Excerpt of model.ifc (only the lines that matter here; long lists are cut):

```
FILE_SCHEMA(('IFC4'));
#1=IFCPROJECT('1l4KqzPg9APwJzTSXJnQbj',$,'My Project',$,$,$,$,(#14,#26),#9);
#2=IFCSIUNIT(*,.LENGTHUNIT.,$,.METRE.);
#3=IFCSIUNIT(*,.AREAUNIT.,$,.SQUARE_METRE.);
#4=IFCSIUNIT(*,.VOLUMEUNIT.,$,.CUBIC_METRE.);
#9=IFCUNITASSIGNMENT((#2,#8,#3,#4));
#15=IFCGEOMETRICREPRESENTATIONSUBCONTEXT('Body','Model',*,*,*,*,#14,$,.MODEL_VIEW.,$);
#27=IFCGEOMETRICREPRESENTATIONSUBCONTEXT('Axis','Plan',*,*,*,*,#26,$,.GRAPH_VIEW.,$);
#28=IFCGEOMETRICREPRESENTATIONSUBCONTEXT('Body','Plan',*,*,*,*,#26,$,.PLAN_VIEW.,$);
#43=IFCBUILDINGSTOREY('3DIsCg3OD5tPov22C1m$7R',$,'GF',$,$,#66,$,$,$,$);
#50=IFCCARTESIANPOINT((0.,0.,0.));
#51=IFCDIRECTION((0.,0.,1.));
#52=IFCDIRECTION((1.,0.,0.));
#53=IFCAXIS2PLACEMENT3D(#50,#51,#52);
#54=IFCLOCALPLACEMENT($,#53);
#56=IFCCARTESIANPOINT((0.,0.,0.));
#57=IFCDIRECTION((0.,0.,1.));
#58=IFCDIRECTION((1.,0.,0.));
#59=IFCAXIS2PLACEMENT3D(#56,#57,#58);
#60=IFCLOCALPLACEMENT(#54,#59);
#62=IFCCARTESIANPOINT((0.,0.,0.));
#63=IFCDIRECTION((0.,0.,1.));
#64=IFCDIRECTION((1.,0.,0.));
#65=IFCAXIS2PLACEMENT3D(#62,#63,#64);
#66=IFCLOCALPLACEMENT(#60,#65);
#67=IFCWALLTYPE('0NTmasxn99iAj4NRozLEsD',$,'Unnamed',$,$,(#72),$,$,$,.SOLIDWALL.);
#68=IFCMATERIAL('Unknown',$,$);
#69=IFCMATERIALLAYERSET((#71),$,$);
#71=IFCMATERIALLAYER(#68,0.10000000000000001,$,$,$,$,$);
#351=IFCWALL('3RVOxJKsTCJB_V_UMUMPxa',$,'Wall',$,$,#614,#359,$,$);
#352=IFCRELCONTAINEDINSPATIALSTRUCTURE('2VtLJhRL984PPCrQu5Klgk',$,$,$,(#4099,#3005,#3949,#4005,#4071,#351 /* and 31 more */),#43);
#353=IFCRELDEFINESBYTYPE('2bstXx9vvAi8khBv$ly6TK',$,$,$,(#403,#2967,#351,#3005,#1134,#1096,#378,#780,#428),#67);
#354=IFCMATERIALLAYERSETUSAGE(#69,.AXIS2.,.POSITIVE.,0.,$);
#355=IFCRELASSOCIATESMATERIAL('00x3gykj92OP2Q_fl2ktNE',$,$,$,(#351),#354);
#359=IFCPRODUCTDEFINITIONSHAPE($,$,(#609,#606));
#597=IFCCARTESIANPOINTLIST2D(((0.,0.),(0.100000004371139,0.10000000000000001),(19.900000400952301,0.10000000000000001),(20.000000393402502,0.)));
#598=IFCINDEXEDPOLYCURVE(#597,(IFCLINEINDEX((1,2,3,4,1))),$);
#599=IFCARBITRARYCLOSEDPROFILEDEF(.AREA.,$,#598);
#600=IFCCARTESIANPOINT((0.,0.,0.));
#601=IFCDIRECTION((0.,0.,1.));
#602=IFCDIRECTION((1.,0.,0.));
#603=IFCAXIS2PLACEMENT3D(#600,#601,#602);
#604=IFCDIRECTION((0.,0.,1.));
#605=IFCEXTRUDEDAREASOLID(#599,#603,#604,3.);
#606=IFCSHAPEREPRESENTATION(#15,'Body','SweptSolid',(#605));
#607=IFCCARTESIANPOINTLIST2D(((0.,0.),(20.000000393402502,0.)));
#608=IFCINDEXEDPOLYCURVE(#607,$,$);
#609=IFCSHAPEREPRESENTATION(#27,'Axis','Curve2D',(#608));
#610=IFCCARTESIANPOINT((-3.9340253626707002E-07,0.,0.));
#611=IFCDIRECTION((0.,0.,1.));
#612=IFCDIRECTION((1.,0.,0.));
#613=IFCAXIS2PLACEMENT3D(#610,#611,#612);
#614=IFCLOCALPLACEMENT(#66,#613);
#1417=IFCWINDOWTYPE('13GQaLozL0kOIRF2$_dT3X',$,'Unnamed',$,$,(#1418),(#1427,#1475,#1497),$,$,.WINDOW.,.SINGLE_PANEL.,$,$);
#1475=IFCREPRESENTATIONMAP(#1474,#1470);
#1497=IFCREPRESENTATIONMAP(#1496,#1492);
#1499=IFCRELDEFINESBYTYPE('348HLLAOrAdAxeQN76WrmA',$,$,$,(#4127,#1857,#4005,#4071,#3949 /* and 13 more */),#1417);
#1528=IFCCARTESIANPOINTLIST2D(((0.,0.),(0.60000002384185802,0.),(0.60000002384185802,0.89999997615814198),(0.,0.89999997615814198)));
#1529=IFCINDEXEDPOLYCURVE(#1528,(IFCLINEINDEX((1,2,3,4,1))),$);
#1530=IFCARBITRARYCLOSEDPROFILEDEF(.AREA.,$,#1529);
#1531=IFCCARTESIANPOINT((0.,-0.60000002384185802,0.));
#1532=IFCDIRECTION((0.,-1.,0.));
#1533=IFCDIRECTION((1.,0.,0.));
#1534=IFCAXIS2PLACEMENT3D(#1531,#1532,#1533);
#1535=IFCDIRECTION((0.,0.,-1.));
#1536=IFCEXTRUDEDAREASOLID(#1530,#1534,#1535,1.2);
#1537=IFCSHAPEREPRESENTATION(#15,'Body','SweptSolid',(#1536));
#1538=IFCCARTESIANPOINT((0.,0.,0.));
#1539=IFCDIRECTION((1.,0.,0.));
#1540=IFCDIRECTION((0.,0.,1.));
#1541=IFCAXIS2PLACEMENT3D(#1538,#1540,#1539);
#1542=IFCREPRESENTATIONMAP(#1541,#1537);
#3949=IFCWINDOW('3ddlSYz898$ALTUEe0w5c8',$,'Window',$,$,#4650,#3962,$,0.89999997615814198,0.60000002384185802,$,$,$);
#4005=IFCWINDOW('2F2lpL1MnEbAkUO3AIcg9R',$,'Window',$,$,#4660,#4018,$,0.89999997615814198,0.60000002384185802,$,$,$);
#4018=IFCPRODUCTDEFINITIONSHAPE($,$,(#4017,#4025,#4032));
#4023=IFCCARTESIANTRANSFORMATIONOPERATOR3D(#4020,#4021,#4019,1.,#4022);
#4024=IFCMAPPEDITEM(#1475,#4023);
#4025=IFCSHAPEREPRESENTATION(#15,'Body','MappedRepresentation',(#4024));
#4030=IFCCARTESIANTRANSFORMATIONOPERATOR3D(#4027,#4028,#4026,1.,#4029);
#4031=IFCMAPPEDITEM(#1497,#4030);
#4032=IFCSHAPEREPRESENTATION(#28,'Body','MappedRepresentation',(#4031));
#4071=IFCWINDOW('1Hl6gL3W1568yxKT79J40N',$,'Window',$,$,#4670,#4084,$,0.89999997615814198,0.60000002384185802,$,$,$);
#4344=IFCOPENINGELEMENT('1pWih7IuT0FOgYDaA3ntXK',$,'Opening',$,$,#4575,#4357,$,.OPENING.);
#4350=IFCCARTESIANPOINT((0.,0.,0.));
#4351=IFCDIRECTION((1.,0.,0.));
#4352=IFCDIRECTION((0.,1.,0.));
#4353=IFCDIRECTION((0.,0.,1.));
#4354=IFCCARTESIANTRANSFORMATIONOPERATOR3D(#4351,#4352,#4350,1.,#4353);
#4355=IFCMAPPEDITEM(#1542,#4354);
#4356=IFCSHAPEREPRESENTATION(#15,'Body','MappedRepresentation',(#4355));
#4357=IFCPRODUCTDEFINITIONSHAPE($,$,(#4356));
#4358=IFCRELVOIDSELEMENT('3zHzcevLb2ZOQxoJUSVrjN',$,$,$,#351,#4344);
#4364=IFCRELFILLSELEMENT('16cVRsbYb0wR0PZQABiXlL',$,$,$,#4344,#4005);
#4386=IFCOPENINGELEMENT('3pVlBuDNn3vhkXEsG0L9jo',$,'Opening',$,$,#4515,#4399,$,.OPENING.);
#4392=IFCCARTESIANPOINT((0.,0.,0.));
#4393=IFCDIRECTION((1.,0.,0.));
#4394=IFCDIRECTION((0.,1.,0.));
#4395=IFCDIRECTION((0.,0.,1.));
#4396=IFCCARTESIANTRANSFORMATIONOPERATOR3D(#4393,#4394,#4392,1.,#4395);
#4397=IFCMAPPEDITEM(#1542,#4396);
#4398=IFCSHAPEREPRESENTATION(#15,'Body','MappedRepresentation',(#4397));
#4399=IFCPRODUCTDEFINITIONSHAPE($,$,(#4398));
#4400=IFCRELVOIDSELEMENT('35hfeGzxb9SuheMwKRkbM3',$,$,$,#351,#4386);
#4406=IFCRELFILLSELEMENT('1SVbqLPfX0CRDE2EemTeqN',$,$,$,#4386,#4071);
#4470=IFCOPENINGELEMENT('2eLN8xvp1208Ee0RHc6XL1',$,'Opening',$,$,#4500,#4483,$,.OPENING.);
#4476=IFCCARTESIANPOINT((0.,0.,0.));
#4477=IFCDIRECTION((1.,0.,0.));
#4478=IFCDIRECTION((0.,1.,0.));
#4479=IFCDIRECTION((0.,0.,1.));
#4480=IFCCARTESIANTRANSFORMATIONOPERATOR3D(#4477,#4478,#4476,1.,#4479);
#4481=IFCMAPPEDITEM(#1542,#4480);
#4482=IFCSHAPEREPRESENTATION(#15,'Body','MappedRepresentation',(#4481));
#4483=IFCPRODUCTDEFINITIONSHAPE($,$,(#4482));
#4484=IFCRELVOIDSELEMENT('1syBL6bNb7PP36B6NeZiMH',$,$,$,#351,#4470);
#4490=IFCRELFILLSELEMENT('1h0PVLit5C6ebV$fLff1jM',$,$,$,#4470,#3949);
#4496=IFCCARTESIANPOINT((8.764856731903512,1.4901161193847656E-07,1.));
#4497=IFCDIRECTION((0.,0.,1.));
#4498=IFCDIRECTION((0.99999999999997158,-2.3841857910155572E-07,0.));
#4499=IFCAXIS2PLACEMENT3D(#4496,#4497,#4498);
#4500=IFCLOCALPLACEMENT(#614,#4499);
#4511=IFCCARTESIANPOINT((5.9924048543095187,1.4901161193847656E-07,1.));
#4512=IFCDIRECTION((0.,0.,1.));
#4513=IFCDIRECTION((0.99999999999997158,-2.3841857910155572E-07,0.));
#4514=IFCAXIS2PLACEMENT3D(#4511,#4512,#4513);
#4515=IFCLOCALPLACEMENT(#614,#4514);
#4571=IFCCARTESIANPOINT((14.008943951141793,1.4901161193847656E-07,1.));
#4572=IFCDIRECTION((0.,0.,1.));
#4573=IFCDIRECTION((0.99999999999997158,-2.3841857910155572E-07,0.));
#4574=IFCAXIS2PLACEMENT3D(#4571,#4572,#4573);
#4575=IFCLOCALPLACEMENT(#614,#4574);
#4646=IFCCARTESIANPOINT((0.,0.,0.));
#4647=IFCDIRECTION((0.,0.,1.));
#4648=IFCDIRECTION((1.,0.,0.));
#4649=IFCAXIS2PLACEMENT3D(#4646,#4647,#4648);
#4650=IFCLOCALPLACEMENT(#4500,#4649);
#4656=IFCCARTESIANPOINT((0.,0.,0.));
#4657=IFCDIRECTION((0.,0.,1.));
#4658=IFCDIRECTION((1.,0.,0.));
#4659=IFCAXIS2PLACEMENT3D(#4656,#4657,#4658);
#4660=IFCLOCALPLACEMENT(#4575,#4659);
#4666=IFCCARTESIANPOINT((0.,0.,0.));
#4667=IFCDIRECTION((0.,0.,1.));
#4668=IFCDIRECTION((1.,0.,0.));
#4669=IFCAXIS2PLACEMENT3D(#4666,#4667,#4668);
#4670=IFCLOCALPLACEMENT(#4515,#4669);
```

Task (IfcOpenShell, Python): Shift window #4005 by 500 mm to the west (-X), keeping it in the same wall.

```python
import ifcopenshell
import ifcopenshell.api.geometry
import ifcopenshell.util.placement
import ifcopenshell.util.unit

model = ifcopenshell.open("model.ifc")
unit_scale = ifcopenshell.util.unit.calculate_unit_scale(model)

window = model.by_id(4005)
opening = window.FillsVoids[0].RelatingOpeningElement
wall = opening.VoidsElements[0].RelatingBuildingElement

wall_matrix = ifcopenshell.util.placement.get_local_placement(wall.ObjectPlacement)
shift = wall_matrix[:3, 0] * -0.5 / unit_scale
before = ifcopenshell.util.placement.get_local_placement(window.ObjectPlacement)[:3, 3].copy()

# The window is placed relative to its opening, so it follows when the opening moves.
matrix = ifcopenshell.util.placement.get_local_placement(opening.ObjectPlacement)
matrix[:3, 3] += shift
ifcopenshell.api.geometry.edit_object_placement(
    model, product=opening, matrix=matrix, is_si=False, should_transform_children=True
)

after = ifcopenshell.util.placement.get_local_placement(window.ObjectPlacement)[:3, 3]
print("window moved by", (after - before).round(3) + 0.0)

model.write("model_updated.ifc")
```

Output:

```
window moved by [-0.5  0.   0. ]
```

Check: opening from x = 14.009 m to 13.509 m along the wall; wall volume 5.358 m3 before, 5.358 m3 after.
